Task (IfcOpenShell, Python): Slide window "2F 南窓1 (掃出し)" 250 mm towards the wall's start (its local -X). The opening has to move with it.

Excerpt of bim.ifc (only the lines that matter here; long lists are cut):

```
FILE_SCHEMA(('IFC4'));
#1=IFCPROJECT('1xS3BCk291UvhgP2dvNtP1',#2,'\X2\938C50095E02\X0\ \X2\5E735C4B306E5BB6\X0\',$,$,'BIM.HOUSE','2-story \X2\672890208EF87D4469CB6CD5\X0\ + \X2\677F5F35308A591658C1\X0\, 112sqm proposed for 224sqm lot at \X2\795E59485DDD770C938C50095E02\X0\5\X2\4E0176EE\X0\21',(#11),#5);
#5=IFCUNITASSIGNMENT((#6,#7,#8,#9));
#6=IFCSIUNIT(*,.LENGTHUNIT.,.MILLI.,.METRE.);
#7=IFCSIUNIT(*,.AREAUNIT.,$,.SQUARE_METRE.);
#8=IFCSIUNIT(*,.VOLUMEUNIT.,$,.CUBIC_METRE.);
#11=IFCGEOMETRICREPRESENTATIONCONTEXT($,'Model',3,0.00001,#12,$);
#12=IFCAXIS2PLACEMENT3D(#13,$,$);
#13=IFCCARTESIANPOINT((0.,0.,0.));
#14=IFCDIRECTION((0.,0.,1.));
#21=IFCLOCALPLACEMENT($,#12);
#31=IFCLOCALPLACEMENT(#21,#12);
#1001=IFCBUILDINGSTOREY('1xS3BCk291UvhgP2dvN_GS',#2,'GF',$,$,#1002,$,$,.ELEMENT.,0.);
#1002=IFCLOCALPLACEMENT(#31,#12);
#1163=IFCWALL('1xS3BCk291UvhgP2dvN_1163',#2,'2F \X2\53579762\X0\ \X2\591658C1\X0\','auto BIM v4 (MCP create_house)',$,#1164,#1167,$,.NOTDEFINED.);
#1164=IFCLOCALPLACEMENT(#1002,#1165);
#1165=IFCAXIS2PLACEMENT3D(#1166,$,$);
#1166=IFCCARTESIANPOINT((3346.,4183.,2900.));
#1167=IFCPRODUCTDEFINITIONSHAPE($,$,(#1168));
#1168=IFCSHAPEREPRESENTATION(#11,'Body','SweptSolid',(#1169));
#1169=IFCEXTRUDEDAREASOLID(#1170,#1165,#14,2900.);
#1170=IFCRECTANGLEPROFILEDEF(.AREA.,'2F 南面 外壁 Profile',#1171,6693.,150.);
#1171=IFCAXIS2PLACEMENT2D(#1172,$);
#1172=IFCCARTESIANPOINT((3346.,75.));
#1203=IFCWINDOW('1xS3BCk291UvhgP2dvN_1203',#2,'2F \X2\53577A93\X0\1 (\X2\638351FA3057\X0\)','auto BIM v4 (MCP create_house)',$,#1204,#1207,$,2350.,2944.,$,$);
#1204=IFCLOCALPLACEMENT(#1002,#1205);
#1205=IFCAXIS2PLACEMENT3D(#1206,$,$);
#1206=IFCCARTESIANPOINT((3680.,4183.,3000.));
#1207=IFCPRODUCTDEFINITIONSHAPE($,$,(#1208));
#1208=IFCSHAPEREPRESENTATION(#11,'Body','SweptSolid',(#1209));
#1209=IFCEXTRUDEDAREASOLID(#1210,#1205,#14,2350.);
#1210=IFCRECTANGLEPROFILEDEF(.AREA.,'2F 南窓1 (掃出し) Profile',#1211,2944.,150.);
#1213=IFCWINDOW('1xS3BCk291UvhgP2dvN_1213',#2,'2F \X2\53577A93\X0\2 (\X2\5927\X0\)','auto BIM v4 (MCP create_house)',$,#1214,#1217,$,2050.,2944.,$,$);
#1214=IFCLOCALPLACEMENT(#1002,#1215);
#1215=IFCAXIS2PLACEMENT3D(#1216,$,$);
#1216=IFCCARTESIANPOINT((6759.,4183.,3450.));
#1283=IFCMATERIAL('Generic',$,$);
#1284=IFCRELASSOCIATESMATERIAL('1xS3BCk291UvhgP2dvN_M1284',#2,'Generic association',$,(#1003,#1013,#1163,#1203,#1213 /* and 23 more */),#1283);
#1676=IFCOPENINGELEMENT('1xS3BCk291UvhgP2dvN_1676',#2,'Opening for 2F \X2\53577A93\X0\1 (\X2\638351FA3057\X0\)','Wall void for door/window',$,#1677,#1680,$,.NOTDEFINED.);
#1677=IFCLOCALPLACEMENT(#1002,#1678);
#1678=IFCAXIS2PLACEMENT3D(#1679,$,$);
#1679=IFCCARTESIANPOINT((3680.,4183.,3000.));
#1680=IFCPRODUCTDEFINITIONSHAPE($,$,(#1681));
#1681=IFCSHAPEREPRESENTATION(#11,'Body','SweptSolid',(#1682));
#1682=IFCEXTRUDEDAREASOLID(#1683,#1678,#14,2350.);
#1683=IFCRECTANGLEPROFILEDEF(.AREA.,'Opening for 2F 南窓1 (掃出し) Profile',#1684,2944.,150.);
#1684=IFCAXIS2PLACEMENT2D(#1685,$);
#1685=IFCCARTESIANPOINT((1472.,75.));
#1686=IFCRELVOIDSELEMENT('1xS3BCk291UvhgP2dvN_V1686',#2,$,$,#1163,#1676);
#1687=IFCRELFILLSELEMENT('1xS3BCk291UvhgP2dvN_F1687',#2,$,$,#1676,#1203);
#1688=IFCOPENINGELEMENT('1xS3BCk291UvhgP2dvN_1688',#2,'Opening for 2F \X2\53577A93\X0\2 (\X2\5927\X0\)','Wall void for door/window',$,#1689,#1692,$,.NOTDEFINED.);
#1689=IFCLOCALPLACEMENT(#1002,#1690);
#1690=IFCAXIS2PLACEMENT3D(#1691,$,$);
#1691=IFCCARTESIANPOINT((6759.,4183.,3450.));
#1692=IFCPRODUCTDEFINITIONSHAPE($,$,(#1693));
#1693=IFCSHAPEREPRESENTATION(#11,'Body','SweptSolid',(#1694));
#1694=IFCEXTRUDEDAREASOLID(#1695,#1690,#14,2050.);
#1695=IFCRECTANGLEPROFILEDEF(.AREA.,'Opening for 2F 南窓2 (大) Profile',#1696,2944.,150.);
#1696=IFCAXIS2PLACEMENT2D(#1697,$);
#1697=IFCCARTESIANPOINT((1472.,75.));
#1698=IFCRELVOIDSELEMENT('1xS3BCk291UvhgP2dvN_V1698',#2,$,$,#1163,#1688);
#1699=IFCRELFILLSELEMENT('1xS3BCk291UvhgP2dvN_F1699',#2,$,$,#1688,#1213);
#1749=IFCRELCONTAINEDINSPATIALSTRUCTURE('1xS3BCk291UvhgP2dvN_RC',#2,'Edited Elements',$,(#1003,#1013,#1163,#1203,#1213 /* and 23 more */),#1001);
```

```python
import ifcopenshell
import ifcopenshell.api.geometry
import ifcopenshell.util.placement

model = ifcopenshell.open("bim.ifc")

window = model.by_guid("1xS3BCk291UvhgP2dvN_1203")
opening = window.FillsVoids[0].RelatingOpeningElement
wall = opening.VoidsElements[0].RelatingBuildingElement

wall_matrix = ifcopenshell.util.placement.get_local_placement(wall.ObjectPlacement)
shift = wall_matrix[:3, 0] * -250.0
before = ifcopenshell.util.placement.get_local_placement(window.ObjectPlacement)[:3, 3].copy()

# The window is not placed relative to its opening, so move both.
for product in (opening, window):
    matrix = ifcopenshell.util.placement.get_local_placement(product.ObjectPlacement)
    matrix[:3, 3] += shift
    ifcopenshell.api.geometry.edit_object_placement(model, product=product, matrix=matrix, is_si=False)

after = ifcopenshell.util.placement.get_local_placement(window.ObjectPlacement)[:3, 3]
print("window moved by", (after - before).round(3) + 0.0)

model.write("bim_rev.ifc")
```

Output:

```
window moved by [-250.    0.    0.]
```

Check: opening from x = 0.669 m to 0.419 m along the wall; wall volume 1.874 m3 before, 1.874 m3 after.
